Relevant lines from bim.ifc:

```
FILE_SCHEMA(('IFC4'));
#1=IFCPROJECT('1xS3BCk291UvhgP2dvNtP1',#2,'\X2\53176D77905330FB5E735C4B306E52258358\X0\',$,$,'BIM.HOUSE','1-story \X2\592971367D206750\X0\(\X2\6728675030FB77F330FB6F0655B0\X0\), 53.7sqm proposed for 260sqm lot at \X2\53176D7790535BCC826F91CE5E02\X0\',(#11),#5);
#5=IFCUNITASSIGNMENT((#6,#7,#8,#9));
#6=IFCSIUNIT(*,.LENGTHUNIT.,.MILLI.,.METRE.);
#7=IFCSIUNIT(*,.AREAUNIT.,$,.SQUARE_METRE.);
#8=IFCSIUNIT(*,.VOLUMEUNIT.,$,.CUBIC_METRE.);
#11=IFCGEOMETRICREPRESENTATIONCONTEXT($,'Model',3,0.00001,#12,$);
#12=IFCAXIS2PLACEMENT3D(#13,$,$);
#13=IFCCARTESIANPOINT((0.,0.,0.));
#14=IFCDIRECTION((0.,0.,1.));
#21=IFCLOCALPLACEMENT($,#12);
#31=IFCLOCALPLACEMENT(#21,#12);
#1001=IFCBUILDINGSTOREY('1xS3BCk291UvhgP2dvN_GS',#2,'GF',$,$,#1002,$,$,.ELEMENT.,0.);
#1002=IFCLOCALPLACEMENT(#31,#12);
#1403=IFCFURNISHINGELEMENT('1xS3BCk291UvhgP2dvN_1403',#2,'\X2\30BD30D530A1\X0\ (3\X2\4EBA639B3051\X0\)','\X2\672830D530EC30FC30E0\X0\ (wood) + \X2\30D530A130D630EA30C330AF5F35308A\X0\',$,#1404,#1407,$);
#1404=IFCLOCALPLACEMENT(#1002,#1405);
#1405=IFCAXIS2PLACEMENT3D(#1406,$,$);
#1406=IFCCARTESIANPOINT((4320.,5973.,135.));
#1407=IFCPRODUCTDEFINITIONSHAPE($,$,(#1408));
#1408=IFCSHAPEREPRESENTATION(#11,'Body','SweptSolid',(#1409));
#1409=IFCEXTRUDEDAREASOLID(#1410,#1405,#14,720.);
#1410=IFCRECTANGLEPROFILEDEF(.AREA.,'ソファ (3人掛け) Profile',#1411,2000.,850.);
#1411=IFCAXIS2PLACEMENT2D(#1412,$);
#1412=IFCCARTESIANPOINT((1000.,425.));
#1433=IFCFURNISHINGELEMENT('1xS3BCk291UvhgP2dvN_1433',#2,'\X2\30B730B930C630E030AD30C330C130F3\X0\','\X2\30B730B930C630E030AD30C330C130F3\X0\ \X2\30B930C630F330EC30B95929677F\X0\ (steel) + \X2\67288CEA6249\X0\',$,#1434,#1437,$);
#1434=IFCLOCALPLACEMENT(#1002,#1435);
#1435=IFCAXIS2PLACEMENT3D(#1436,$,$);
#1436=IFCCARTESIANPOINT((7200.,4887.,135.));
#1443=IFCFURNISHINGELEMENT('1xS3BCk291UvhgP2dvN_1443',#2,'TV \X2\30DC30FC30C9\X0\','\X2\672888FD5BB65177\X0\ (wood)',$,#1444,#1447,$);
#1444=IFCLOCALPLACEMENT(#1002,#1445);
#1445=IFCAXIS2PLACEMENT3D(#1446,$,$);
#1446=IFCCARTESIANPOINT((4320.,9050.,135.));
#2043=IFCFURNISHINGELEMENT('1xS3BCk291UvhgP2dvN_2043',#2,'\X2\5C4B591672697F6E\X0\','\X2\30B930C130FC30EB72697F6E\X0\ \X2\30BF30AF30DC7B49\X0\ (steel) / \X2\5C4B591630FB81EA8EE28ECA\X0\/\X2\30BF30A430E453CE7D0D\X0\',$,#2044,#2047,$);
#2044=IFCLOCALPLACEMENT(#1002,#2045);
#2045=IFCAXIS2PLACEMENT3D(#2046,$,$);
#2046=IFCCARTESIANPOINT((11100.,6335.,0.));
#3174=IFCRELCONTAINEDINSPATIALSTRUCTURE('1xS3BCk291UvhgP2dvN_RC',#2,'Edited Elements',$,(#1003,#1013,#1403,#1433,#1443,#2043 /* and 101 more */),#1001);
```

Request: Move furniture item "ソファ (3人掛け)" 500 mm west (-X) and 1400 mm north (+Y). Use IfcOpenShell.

```python
import ifcopenshell
import ifcopenshell.api.geometry
import ifcopenshell.util.placement

model = ifcopenshell.open("bim.ifc")

item = model.by_guid("1xS3BCk291UvhgP2dvN_1403")
matrix = ifcopenshell.util.placement.get_local_placement(item.ObjectPlacement)
matrix[0, 3] -= 500.0
matrix[1, 3] += 1400.0
ifcopenshell.api.geometry.edit_object_placement(model, product=item, matrix=matrix, is_si=False)

print(ifcopenshell.util.placement.get_local_placement(item.ObjectPlacement).round(3) + 0.0)

model.write("bim_updated.ifc")
```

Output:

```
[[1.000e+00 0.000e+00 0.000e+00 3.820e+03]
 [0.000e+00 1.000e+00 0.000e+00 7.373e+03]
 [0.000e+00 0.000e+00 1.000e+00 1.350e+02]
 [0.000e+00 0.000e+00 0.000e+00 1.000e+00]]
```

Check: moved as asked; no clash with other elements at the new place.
